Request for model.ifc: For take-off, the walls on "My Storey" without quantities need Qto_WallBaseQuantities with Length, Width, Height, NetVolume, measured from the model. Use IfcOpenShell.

First a look at what the model holds.

```python
import ifcopenshell
import ifcopenshell.util.element
import ifcopenshell.util.unit

model = ifcopenshell.open("model.ifc")
print(model.schema)
for unit_type in ("LENGTHUNIT", "AREAUNIT", "VOLUMEUNIT"):
    print(unit_type, ifcopenshell.util.unit.calculate_unit_scale(model, unit_type))
storey = next(s for s in model.by_type("IfcBuildingStorey") if s.Name == "My Storey")
walls = [e for e in ifcopenshell.util.element.get_decomposition(storey) if e.is_a("IfcWall")]
for e in sorted(walls, key=lambda e: e.id()):
    print(e.id(), e.is_a(), e.Name, list(ifcopenshell.util.element.get_psets(e, qtos_only=True)), sep=" | ")
```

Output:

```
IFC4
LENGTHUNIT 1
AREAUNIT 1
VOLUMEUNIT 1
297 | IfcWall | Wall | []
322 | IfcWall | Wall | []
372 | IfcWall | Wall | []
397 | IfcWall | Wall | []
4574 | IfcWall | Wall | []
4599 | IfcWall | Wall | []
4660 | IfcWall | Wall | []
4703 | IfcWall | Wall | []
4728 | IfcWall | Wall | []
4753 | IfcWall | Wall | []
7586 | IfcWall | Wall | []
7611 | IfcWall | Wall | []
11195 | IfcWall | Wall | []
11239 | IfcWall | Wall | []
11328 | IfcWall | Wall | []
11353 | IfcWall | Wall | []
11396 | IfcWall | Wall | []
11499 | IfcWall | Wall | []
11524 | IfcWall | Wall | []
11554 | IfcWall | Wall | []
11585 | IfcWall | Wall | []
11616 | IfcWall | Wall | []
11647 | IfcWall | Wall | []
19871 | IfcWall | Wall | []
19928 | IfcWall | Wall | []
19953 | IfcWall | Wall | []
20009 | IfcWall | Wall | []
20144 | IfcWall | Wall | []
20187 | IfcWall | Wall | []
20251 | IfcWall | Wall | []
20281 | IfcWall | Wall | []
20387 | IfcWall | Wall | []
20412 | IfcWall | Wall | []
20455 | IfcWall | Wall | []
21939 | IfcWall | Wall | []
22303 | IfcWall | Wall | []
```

```python
import ifcopenshell
import ifcopenshell.api.pset
import ifcopenshell.geom
import ifcopenshell.util.element
import ifcopenshell.util.shape
import ifcopenshell.util.unit

model = ifcopenshell.open("model.ifc")
unit_scale = ifcopenshell.util.unit.calculate_unit_scale(model)
volume_scale = ifcopenshell.util.unit.calculate_unit_scale(model, "VOLUMEUNIT")
settings = ifcopenshell.geom.settings()

storey = next(s for s in model.by_type("IfcBuildingStorey") if s.Name == "My Storey")
walls = [e for e in ifcopenshell.util.element.get_decomposition(storey) if e.is_a("IfcWall")]

for e in sorted(walls, key=lambda e: e.id()):
    if ifcopenshell.util.element.get_psets(e, qtos_only=True, should_inherit=False):
        continue
    # Geometry comes back in metres, in the element's own axes.
    shape = ifcopenshell.geom.create_shape(settings, e)
    values = {
        "Length": ifcopenshell.util.shape.get_x(shape.geometry) / unit_scale,
        "Width": ifcopenshell.util.shape.get_y(shape.geometry) / unit_scale,
        "Height": ifcopenshell.util.shape.get_z(shape.geometry) / unit_scale,
        "NetVolume": ifcopenshell.util.shape.get_volume(shape.geometry) / volume_scale,
    }
    qto = ifcopenshell.api.pset.add_qto(model, product=e, name="Qto_WallBaseQuantities")
    ifcopenshell.api.pset.edit_qto(model, qto=qto, properties=values)
    print(e.id(), {k: round(v, 3) for k, v in values.items()})

model.write("model_v2.ifc")
```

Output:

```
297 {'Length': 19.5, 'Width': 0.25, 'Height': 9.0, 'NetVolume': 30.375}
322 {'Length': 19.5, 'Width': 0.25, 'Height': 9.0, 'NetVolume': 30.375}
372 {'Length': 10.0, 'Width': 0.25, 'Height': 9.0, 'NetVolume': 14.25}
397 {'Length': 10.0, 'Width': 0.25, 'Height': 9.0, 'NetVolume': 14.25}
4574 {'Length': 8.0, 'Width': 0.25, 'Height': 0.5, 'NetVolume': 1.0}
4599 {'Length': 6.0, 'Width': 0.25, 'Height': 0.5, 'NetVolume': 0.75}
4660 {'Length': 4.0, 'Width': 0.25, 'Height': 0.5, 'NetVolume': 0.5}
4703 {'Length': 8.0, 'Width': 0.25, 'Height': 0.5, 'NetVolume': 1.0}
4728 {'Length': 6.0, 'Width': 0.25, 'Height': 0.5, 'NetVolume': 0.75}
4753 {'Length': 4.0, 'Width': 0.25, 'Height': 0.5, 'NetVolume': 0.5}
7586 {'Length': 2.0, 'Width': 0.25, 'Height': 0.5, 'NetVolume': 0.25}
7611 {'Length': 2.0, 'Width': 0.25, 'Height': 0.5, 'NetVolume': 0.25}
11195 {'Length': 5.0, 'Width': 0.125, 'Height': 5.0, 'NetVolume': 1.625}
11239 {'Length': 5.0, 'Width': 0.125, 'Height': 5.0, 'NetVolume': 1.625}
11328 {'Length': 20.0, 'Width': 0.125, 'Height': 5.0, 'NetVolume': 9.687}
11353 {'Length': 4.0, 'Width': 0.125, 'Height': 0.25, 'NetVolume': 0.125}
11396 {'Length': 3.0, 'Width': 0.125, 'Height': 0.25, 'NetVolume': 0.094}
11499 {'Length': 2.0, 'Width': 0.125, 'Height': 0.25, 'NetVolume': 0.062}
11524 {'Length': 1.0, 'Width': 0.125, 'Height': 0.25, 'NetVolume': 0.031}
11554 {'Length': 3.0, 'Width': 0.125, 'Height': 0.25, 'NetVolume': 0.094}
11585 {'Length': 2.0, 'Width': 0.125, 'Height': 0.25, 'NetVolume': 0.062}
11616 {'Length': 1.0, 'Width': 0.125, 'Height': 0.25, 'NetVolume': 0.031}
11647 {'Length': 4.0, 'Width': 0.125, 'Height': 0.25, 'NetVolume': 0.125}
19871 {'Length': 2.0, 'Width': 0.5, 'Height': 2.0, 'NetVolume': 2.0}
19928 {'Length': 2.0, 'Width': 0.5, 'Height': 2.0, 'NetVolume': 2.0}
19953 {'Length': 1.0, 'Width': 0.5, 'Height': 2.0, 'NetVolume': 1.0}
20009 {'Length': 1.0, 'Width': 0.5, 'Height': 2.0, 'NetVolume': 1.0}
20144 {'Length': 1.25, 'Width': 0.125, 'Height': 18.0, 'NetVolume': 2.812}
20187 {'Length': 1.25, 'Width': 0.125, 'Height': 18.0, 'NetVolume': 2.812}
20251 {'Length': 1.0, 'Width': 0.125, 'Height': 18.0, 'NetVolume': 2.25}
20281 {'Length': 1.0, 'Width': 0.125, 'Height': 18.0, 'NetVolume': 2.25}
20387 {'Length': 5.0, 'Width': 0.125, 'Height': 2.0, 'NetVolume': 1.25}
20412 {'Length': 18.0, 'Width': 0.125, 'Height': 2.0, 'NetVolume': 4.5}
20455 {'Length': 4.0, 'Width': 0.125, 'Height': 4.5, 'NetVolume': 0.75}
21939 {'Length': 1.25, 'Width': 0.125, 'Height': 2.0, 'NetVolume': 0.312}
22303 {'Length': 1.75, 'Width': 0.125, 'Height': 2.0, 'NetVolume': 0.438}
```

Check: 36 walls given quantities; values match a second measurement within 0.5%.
